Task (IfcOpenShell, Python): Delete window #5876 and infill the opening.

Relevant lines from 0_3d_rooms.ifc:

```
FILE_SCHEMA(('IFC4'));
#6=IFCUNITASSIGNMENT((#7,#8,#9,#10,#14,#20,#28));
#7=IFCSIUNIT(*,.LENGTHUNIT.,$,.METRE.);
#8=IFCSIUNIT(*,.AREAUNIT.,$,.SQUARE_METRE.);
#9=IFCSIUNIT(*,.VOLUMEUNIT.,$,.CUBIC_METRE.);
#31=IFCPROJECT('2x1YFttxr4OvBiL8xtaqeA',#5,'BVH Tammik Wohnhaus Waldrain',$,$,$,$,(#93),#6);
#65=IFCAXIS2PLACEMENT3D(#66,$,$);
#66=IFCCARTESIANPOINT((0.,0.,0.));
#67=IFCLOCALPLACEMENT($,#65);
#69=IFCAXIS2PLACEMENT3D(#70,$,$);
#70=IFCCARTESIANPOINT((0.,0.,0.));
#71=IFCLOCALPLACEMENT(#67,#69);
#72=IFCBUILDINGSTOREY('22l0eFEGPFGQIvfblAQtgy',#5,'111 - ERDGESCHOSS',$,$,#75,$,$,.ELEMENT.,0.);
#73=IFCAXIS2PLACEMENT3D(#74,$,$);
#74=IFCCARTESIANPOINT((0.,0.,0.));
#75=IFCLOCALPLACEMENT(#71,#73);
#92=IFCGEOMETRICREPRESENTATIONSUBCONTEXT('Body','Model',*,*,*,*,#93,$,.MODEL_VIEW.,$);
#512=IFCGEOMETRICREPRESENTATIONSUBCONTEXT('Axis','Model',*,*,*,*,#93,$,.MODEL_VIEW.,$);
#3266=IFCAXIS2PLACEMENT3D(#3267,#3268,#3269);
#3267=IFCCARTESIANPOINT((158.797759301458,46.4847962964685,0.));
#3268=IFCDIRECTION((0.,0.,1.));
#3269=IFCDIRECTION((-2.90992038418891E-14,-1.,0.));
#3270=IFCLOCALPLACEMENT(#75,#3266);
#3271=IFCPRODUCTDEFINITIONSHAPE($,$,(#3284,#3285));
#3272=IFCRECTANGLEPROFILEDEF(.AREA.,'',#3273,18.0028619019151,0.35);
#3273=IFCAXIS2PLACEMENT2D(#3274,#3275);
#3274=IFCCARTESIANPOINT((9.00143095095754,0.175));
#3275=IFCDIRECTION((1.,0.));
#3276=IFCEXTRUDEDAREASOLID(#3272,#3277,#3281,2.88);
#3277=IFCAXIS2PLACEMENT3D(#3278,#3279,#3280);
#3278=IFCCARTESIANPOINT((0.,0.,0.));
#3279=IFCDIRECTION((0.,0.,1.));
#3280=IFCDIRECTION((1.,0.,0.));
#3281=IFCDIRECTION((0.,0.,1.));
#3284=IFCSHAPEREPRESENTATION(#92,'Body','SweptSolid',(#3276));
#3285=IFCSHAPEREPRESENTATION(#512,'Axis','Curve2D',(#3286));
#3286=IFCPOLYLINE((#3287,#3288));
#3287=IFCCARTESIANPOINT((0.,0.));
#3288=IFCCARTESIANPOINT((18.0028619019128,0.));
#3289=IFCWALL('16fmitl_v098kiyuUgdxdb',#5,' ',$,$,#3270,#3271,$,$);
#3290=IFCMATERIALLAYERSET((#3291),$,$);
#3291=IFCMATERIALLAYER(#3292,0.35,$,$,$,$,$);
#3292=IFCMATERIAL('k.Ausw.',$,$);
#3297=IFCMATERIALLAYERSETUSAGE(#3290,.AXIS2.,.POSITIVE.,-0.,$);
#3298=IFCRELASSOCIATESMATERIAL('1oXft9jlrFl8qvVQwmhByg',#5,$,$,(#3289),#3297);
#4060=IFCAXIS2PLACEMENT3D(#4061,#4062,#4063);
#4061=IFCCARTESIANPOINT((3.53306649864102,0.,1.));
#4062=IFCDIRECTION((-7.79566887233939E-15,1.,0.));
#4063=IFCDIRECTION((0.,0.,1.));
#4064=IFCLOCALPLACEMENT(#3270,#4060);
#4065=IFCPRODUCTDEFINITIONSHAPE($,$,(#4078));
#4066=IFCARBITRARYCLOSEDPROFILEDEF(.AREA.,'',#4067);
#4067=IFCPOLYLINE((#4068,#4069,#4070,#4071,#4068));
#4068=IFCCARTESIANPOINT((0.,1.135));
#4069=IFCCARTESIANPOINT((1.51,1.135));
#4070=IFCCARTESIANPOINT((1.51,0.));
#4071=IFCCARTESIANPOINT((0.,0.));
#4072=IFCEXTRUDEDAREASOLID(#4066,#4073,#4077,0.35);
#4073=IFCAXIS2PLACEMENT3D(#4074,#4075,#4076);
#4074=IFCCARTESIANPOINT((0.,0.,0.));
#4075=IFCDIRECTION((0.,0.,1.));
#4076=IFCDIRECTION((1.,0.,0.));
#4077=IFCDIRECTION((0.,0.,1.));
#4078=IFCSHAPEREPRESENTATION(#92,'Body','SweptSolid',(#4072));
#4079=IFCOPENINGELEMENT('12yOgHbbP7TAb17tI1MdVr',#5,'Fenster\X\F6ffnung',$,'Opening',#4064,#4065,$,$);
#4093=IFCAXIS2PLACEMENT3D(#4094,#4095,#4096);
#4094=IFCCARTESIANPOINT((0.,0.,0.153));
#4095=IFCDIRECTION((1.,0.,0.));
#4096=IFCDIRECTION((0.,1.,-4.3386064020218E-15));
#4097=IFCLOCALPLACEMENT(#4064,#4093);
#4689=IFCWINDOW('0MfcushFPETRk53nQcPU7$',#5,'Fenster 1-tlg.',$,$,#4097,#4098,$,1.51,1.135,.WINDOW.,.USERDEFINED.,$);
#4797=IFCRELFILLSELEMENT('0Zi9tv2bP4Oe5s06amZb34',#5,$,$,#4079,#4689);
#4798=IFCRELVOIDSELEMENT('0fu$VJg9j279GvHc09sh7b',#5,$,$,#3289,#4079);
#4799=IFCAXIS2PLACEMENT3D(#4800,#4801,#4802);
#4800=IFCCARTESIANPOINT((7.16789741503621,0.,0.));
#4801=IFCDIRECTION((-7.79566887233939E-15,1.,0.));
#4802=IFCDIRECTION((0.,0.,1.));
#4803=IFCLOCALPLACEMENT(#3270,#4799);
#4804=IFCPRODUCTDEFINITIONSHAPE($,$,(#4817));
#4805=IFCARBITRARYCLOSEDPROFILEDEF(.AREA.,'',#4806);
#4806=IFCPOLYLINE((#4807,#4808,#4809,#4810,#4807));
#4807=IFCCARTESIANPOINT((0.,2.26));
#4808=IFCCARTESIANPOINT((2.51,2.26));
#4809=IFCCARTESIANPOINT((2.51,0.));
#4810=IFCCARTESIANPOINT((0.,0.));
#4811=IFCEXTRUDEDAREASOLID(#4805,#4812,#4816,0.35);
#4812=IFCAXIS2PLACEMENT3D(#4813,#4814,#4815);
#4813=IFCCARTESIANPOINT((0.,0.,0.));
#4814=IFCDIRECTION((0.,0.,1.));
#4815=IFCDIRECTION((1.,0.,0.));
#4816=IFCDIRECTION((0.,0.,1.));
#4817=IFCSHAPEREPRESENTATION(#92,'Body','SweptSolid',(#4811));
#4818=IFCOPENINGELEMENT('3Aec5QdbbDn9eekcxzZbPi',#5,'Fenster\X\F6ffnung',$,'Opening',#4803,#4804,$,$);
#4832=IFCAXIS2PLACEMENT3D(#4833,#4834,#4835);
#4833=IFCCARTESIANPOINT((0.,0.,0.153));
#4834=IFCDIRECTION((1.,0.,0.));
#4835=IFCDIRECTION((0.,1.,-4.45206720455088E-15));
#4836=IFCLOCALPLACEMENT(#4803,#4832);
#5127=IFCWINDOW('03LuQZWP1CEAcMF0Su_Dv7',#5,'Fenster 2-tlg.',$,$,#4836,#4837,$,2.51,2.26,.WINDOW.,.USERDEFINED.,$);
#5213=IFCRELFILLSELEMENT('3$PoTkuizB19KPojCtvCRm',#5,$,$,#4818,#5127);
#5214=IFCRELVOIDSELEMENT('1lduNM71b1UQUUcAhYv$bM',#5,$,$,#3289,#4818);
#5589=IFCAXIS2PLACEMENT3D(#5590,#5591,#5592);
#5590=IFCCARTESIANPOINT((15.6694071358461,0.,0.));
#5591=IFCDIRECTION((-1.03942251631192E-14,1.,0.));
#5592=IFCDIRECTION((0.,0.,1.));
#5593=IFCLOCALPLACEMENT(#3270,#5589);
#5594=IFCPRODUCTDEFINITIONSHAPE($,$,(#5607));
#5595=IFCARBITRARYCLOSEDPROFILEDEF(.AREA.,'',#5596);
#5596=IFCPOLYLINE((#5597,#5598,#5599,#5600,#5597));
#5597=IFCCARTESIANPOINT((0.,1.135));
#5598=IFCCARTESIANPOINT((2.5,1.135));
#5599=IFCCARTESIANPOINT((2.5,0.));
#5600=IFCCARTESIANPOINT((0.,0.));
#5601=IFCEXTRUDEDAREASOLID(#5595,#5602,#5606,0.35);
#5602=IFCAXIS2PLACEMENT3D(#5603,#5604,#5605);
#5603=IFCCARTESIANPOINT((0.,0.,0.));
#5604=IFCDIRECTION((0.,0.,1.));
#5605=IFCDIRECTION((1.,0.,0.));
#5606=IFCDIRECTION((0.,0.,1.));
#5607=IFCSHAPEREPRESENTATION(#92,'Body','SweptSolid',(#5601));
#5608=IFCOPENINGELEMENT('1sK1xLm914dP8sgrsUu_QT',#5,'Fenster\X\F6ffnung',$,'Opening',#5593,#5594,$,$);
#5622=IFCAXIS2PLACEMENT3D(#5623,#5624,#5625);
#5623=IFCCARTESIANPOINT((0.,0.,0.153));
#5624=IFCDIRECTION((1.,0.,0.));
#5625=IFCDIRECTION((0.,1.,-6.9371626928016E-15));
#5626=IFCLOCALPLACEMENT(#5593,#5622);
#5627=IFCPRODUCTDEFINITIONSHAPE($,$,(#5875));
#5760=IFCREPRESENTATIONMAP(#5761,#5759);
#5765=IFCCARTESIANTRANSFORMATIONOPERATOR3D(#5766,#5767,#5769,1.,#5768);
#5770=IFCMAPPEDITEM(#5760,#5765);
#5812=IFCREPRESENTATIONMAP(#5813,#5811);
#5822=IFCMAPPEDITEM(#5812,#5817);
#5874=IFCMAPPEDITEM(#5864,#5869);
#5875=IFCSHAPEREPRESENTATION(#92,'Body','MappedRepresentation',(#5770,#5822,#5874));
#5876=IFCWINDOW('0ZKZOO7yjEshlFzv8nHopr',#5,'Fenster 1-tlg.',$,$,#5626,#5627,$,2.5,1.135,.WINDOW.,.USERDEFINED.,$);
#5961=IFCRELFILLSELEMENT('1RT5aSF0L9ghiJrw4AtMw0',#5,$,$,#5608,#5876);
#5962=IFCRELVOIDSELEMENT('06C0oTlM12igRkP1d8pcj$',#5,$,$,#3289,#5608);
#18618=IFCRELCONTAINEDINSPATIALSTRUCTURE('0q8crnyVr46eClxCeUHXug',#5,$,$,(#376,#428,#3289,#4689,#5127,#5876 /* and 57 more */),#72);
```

```python
import ifcopenshell
import ifcopenshell.api.feature
import ifcopenshell.api.root
import ifcopenshell.geom
import ifcopenshell.util.shape

model = ifcopenshell.open("0_3d_rooms.ifc")
settings = ifcopenshell.geom.settings()


def volume(element):
    """Net volume in cubic metres, openings subtracted."""
    shape = ifcopenshell.geom.create_shape(settings, element)
    return ifcopenshell.util.shape.get_volume(shape.geometry)


window = model.by_guid("0ZKZOO7yjEshlFzv8nHopr")
opening = window.FillsVoids[0].RelatingOpeningElement
wall = opening.VoidsElements[0].RelatingBuildingElement
before = volume(wall)

ifcopenshell.api.root.remove_product(model, product=window)
ifcopenshell.api.feature.remove_feature(model, feature=opening)

after = volume(wall)

print(f"wall volume {before:.3f} -> {after:.3f} m3")

model.write("0_3d_rooms_updated.ifc")
```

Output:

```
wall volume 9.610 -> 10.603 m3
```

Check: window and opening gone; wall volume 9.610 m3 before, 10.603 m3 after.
